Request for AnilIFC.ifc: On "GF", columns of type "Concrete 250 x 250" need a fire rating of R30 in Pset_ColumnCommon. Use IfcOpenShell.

First a look at what the model holds.

```python
import ifcopenshell
import ifcopenshell.util.element

model = ifcopenshell.open("AnilIFC.ifc")
print(model.schema)
storey = next(s for s in model.by_type("IfcBuildingStorey") if s.Name == "GF")
columns = [e for e in ifcopenshell.util.element.get_decomposition(storey) if e.is_a("IfcColumn")]
seen = {}
for e in columns:
    element_type = ifcopenshell.util.element.get_type(e)
    key = (element_type.Name if element_type != e and element_type else None, ifcopenshell.util.element.get_pset(e, "Pset_ColumnCommon", "FireRating"))
    seen[key] = seen.get(key, 0) + 1
for (name, value), count in sorted(seen.items(), key=str):
    print(count, "x", name, "|", value)
```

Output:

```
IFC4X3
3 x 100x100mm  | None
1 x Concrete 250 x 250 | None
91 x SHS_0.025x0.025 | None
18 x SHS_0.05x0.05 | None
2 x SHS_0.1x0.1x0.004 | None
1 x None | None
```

```python
import ifcopenshell
import ifcopenshell.api.pset
import ifcopenshell.util.element

model = ifcopenshell.open("AnilIFC.ifc")

storey = next(s for s in model.by_type("IfcBuildingStorey") if s.Name == "GF")
columns = [e for e in ifcopenshell.util.element.get_decomposition(storey) if e.is_a("IfcColumn")]

count = 0
for e in columns:
    element_type = ifcopenshell.util.element.get_type(e)
    if element_type in (None, e) or element_type.Name != "Concrete 250 x 250":
        continue
    # add_pset returns the element's existing set when there is one.
    pset = ifcopenshell.api.pset.add_pset(model, product=e, name="Pset_ColumnCommon")
    ifcopenshell.api.pset.edit_pset(model, pset=pset, properties={"FireRating": "R30"})
    count += 1

print(count, "columns updated")

model.write("AnilIFC_rev.ifc")
```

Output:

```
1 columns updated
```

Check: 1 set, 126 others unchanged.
